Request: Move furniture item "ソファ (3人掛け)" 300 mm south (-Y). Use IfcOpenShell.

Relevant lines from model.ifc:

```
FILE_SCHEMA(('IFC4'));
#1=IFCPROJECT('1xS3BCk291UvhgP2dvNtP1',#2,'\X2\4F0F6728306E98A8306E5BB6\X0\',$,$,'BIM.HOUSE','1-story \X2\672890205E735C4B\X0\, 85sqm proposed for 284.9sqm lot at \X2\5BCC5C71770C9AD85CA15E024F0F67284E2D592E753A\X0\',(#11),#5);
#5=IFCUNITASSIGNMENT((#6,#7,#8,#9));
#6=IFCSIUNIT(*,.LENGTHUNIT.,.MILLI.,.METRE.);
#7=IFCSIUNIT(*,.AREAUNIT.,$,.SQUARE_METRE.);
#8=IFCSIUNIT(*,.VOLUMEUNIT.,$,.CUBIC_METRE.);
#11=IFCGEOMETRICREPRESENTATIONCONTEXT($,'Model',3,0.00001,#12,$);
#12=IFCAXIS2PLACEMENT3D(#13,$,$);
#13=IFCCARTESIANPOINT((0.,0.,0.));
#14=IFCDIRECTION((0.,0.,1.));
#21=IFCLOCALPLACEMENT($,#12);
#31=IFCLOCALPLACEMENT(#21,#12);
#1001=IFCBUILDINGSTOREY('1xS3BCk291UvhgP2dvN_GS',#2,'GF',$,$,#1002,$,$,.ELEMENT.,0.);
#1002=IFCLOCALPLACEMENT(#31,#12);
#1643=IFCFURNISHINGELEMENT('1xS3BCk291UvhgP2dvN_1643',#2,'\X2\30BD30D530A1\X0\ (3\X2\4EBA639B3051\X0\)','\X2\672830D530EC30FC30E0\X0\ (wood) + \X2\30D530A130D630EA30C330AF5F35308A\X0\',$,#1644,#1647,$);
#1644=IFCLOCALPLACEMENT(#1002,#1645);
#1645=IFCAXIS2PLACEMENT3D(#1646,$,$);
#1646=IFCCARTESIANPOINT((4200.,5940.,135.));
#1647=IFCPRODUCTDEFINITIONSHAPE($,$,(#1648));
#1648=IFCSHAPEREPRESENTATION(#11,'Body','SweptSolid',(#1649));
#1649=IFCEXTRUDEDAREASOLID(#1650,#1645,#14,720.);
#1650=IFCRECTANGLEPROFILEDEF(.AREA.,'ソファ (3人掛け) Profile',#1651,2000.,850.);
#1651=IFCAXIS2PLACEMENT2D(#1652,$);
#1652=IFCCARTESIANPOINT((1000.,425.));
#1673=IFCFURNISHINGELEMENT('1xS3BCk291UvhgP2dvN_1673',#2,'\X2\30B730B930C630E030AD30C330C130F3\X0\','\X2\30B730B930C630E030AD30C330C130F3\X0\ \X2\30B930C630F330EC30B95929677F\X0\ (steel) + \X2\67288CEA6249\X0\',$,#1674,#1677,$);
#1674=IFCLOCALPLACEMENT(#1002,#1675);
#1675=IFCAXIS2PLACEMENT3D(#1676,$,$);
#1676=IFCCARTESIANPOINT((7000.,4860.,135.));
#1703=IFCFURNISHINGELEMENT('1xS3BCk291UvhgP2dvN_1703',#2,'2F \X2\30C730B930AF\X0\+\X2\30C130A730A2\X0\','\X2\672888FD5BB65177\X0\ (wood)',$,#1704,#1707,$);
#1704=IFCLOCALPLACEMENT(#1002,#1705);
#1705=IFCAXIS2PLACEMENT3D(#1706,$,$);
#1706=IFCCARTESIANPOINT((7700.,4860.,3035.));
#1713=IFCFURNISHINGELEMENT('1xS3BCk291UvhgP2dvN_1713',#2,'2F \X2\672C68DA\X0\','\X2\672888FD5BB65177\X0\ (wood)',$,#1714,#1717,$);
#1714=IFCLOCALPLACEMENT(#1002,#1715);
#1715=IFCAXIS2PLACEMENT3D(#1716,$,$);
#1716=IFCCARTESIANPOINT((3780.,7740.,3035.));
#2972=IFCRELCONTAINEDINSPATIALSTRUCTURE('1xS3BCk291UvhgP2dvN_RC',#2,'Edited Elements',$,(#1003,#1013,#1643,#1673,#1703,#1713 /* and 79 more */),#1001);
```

```python
import ifcopenshell
import ifcopenshell.api.geometry
import ifcopenshell.util.placement
import ifcopenshell.util.unit

model = ifcopenshell.open("model.ifc")
unit_scale = ifcopenshell.util.unit.calculate_unit_scale(model)

item = model.by_id(1643)
matrix = ifcopenshell.util.placement.get_local_placement(item.ObjectPlacement)
matrix[1, 3] -= 0.3 / unit_scale
ifcopenshell.api.geometry.edit_object_placement(model, product=item, matrix=matrix, is_si=False)

print(ifcopenshell.util.placement.get_local_placement(item.ObjectPlacement).round(3) + 0.0)

model.write("model_updated.ifc")
```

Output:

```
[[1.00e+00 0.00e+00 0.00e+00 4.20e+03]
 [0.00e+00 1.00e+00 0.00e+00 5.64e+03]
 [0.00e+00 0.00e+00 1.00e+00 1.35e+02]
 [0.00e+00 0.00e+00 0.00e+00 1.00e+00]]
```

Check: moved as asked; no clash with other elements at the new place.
